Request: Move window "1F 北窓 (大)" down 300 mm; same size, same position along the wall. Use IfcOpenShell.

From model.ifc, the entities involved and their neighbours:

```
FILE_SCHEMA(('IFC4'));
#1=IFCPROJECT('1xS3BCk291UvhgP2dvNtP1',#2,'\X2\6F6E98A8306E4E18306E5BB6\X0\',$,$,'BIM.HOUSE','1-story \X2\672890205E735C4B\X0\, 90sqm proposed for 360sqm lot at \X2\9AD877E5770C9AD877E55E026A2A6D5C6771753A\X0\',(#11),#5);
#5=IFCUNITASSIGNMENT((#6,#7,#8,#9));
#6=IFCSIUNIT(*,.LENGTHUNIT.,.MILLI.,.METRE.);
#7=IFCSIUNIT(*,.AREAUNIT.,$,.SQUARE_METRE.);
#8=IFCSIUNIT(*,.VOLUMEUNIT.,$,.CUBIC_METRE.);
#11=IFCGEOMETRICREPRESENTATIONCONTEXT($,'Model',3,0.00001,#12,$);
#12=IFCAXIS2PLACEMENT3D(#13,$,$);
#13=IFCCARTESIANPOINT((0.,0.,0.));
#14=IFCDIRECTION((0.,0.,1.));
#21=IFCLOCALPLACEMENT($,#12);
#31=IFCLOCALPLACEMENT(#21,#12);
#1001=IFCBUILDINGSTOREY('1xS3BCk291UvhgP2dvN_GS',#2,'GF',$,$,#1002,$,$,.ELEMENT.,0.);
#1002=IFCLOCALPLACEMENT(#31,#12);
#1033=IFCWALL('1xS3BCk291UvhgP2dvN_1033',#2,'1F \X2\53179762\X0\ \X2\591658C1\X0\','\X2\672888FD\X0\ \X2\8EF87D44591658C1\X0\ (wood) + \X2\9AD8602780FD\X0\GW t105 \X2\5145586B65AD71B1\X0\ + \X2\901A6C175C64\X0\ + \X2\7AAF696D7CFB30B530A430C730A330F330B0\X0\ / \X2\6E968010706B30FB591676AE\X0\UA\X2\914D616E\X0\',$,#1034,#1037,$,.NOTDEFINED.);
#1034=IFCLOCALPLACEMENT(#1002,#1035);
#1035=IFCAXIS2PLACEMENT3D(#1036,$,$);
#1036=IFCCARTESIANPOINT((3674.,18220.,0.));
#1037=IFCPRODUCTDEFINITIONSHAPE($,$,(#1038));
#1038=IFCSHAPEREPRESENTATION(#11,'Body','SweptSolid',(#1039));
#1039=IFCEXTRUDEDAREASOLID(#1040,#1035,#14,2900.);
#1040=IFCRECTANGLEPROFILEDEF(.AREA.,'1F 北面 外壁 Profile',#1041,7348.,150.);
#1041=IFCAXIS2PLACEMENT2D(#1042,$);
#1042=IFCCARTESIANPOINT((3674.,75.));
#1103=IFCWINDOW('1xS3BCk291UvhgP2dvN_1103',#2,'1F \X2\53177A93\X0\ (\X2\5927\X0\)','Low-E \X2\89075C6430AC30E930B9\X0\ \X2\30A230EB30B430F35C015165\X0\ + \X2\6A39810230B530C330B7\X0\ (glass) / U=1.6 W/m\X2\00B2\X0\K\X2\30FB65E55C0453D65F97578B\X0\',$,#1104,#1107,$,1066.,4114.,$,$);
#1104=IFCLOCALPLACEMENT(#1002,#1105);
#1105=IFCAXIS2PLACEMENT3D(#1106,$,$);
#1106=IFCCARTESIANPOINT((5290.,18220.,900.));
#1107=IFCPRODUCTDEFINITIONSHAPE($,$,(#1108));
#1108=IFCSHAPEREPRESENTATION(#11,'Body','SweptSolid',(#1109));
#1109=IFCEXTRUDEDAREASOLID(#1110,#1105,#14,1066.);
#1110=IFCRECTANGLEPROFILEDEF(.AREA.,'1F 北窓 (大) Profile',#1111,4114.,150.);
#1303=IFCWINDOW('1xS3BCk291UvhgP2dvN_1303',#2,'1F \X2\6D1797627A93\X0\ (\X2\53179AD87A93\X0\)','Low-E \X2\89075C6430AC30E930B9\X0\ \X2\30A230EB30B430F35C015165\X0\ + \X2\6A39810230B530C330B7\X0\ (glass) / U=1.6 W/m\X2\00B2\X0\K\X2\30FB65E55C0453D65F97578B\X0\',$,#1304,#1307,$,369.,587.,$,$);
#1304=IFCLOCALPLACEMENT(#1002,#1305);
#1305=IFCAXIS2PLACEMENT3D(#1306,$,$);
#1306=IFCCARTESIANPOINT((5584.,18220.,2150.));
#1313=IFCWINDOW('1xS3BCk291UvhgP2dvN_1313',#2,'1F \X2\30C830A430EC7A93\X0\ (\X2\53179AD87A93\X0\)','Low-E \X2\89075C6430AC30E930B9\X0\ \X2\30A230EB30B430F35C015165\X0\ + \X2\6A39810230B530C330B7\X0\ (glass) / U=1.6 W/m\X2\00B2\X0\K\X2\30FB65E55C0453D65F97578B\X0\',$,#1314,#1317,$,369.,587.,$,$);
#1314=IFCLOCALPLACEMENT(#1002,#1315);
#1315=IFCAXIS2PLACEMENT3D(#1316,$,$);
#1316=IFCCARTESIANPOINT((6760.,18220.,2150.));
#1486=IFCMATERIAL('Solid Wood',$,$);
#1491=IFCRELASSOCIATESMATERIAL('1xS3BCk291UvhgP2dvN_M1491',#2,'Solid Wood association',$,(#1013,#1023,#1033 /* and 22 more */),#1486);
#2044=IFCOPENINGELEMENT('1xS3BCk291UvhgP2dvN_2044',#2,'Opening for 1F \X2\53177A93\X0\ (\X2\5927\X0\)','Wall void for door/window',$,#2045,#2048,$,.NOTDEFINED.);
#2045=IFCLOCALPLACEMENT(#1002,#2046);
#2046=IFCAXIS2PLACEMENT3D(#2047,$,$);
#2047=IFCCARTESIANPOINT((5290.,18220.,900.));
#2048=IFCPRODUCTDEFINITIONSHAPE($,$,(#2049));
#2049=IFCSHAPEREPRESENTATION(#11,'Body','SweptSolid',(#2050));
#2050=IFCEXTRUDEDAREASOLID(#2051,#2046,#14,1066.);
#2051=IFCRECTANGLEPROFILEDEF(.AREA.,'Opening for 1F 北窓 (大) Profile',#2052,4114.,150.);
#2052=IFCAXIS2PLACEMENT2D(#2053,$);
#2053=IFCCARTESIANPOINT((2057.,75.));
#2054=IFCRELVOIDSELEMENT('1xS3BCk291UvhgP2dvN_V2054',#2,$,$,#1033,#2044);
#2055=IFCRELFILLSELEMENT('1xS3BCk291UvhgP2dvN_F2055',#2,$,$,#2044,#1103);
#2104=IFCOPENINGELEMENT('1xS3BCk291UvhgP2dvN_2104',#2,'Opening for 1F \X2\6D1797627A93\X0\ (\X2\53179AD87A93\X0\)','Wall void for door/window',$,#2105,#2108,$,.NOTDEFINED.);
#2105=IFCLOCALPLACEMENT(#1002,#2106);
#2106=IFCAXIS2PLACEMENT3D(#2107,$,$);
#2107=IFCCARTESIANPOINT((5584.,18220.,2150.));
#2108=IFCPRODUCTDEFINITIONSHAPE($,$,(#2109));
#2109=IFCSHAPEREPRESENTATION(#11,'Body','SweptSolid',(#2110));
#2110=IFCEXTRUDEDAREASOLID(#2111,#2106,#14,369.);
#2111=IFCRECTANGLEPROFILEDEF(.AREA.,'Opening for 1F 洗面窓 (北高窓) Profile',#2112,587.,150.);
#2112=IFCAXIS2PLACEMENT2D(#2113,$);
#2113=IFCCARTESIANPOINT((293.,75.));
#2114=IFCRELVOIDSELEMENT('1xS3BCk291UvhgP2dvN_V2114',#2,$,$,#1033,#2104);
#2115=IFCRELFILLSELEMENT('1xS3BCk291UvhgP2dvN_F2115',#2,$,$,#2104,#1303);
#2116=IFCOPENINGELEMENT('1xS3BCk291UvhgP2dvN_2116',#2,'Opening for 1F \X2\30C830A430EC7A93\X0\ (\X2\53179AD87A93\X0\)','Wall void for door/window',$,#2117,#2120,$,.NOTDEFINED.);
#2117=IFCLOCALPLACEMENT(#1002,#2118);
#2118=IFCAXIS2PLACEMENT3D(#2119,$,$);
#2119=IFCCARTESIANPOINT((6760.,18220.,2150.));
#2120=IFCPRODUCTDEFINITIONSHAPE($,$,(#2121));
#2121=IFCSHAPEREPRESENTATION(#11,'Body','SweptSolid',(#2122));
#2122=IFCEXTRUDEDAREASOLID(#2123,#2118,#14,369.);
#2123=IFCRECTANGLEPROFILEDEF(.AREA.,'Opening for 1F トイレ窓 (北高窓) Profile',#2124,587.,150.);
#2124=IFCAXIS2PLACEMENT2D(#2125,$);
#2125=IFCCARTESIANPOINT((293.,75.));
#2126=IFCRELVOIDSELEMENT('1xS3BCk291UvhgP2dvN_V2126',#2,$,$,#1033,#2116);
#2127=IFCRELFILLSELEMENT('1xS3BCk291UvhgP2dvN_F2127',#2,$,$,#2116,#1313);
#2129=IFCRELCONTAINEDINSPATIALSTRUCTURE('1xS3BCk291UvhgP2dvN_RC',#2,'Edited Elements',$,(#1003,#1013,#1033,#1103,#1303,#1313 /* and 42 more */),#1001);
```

```python
import numpy as np
import ifcopenshell
import ifcopenshell.api.geometry
import ifcopenshell.util.placement
import ifcopenshell.util.unit

model = ifcopenshell.open("model.ifc")
unit_scale = ifcopenshell.util.unit.calculate_unit_scale(model)

window = model.by_guid("1xS3BCk291UvhgP2dvN_1103")
opening = window.FillsVoids[0].RelatingOpeningElement
dz = -300.0

shift = np.array([0.0, 0.0, dz])
# The window is not placed relative to its opening, so move both.
for product in (opening, window):
    matrix = ifcopenshell.util.placement.get_local_placement(product.ObjectPlacement)
    matrix[:3, 3] += shift
    ifcopenshell.api.geometry.edit_object_placement(model, product=product, matrix=matrix, is_si=False)

print(f"moved by {dz * unit_scale:+.3f} m")

model.write("model_rev.ifc")
```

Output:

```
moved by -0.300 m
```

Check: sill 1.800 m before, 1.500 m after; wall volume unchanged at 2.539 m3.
